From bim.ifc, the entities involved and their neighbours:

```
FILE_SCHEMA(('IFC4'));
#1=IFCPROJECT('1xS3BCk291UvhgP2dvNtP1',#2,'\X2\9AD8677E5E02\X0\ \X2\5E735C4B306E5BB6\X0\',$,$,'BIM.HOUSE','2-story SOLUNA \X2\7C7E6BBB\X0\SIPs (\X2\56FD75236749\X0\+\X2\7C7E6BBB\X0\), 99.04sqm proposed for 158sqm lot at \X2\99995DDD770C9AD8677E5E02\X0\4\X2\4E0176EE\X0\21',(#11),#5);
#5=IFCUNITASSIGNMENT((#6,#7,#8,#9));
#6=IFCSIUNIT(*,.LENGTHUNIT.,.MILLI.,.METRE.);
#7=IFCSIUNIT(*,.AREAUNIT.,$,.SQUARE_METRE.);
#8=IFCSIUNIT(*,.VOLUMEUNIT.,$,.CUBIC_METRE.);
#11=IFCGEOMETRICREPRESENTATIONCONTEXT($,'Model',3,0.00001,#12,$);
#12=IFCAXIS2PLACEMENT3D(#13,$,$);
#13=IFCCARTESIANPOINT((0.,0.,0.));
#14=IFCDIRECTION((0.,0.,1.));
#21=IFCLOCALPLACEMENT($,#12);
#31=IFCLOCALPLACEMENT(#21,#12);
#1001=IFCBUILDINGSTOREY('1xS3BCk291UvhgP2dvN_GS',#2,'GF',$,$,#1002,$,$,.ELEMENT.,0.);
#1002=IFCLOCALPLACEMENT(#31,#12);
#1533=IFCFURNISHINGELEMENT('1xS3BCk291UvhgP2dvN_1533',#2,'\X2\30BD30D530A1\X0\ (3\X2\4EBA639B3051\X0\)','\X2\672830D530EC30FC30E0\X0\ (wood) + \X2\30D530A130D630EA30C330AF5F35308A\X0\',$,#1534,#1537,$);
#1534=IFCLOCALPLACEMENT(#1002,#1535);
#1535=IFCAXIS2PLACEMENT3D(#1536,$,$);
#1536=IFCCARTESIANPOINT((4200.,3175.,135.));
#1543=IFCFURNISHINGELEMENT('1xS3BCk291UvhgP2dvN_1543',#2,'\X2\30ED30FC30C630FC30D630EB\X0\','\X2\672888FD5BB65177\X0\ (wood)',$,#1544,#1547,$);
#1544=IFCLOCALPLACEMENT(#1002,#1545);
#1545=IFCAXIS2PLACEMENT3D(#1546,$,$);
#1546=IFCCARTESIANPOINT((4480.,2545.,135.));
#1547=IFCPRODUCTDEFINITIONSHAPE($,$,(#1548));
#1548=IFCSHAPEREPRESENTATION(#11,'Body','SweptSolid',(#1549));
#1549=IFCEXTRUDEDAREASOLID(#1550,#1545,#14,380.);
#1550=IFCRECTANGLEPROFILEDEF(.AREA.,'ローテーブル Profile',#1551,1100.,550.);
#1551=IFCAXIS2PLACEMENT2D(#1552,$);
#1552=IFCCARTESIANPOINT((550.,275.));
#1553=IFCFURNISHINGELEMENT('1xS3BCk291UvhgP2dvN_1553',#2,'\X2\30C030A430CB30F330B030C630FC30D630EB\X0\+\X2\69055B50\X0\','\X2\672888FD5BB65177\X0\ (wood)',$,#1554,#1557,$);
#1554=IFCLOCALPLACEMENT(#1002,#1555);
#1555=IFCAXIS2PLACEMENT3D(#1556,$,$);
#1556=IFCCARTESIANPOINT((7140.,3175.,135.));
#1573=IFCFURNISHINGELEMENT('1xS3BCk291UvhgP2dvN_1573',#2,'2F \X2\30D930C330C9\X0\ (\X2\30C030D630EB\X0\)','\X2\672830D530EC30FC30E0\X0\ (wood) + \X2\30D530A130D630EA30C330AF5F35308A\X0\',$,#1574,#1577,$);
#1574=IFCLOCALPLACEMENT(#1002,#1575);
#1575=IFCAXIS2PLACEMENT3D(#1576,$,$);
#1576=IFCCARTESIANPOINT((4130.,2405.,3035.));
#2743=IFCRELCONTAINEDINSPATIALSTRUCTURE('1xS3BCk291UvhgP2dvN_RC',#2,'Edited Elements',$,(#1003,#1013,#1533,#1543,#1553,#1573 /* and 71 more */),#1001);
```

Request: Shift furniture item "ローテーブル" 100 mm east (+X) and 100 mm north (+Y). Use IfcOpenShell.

```python
import ifcopenshell
import ifcopenshell.api.geometry
import ifcopenshell.util.placement
import ifcopenshell.util.unit

model = ifcopenshell.open("bim.ifc")
unit_scale = ifcopenshell.util.unit.calculate_unit_scale(model)

item = model.by_guid("1xS3BCk291UvhgP2dvN_1543")
matrix = ifcopenshell.util.placement.get_local_placement(item.ObjectPlacement)
matrix[0, 3] += 0.1 / unit_scale
matrix[1, 3] += 0.1 / unit_scale
ifcopenshell.api.geometry.edit_object_placement(model, product=item, matrix=matrix, is_si=False)

print(ifcopenshell.util.placement.get_local_placement(item.ObjectPlacement).round(3) + 0.0)

model.write("bim_rev.ifc")
```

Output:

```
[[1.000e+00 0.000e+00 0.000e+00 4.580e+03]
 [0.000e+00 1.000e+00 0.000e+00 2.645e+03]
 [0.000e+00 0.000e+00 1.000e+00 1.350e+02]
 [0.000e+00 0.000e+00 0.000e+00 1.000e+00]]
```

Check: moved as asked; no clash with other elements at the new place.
